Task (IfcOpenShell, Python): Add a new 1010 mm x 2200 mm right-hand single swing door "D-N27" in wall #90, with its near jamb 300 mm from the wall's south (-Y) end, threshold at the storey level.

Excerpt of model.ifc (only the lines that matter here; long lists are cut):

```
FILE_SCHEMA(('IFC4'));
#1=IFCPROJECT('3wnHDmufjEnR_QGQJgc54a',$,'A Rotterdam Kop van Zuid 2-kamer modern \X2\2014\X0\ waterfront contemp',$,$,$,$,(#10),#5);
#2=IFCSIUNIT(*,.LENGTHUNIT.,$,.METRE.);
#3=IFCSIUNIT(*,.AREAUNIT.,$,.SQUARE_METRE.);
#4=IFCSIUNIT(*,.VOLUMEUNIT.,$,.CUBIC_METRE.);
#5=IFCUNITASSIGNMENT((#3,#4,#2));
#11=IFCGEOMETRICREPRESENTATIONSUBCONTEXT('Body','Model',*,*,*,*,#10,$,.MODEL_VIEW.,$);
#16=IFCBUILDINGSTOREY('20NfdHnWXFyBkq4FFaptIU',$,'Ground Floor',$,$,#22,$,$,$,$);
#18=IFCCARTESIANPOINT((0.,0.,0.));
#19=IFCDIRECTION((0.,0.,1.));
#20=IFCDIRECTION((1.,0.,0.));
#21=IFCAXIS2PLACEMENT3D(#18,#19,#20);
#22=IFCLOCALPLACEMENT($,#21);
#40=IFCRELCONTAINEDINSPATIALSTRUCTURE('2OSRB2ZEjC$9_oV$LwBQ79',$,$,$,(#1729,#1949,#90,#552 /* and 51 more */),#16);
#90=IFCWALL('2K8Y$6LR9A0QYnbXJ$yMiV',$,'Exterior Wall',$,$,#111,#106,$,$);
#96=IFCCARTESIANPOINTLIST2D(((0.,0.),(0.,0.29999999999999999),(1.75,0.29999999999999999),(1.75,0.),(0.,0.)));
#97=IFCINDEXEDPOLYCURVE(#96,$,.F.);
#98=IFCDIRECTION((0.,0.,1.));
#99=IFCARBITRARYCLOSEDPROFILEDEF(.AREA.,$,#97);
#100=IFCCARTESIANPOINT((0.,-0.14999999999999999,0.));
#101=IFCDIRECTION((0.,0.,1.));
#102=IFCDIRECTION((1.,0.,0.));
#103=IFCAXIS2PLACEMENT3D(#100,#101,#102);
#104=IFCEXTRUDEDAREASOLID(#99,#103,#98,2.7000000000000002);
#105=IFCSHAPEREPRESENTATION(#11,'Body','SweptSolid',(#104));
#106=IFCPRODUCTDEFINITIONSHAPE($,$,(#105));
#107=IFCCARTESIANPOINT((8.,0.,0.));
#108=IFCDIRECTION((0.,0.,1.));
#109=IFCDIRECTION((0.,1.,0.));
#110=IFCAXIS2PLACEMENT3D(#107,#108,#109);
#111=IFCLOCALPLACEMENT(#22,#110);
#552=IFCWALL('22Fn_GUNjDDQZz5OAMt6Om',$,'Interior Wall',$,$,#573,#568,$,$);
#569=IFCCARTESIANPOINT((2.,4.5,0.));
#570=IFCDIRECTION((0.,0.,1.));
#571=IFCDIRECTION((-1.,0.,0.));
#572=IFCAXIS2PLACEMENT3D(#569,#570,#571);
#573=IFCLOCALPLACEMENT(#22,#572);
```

```python
import numpy as np
import ifcopenshell
import ifcopenshell.api.feature
import ifcopenshell.api.geometry
import ifcopenshell.api.root
import ifcopenshell.api.spatial
import ifcopenshell.geom
import ifcopenshell.util.element
import ifcopenshell.util.placement
import ifcopenshell.util.representation
import ifcopenshell.util.shape
import ifcopenshell.util.unit

model = ifcopenshell.open("model.ifc")
unit_scale = ifcopenshell.util.unit.calculate_unit_scale(model)
settings = ifcopenshell.geom.settings()


def volume(element):
    """Net volume in cubic metres, openings subtracted."""
    shape = ifcopenshell.geom.create_shape(settings, element)
    return ifcopenshell.util.shape.get_volume(shape.geometry)


wall = model.by_guid("2K8Y$6LR9A0QYnbXJ$yMiV")
storey = ifcopenshell.util.element.get_container(wall, ifc_class="IfcBuildingStorey")
context = ifcopenshell.util.representation.get_context(model, "Model", "Body", "MODEL_VIEW")
before = volume(wall)

width, height, from_end, sill = 1.01, 2.2, 0.3, 0.0  # metres

# The wall runs along its own X axis, and the end named is its -X end.
wall_shape = ifcopenshell.geom.create_shape(settings, wall)
x, y, z = ifcopenshell.util.shape.get_vertices(wall_shape.geometry).T
start = x.min() + from_end
face, thickness = float(y.min()), float(y.max() - y.min())
wall_matrix = ifcopenshell.util.placement.get_local_placement(wall.ObjectPlacement)
level = ifcopenshell.util.placement.get_local_placement(storey.ObjectPlacement)[2, 3]


def in_wall(x, y):
    """Placement at x, y metres in the wall's axes, at sill height."""
    matrix = wall_matrix.copy()
    matrix[:, 3] = wall_matrix @ np.array([x / unit_scale, y / unit_scale, 0.0, 1.0])
    matrix[2, 3] = level + sill / unit_scale
    return matrix


# Opening: a box that overshoots both wall faces by 50 mm.
opening = ifcopenshell.api.root.create_entity(model, ifc_class="IfcOpeningElement", predefined_type="OPENING")
box = ifcopenshell.api.geometry.add_wall_representation(
    model, context=context, length=width, height=height, thickness=thickness + 0.1
)
ifcopenshell.api.geometry.assign_representation(model, product=opening, representation=box)
ifcopenshell.api.geometry.edit_object_placement(model, product=opening, matrix=in_wall(start, face - 0.05), is_si=False)
ifcopenshell.api.feature.add_feature(model, feature=opening, element=wall)

door = ifcopenshell.api.root.create_entity(model, ifc_class="IfcDoor", name="D-N27", predefined_type="DOOR")
door.OverallWidth, door.OverallHeight = width / unit_scale, height / unit_scale
door.OperationType = "SINGLE_SWING_RIGHT"
body = ifcopenshell.api.geometry.add_door_representation(
    model,
    context=context,
    overall_width=door.OverallWidth,
    overall_height=door.OverallHeight,
    operation_type="SINGLE_SWING_RIGHT",
    lining_properties={"LiningDepth": thickness / unit_scale, "ThresholdDepth": thickness / unit_scale},
)
ifcopenshell.api.geometry.assign_representation(model, product=door, representation=body)
ifcopenshell.api.spatial.assign_container(model, products=[door], relating_structure=storey)
ifcopenshell.api.feature.add_filling(model, opening=opening, element=door)

# The lining spans the wall, so the door starts at the wall face.
ifcopenshell.api.geometry.edit_object_placement(model, product=door, matrix=in_wall(start, face), is_si=False)

after = volume(wall)

print(f"wall volume {before:.3f} -> {after:.3f} m3")

model.write("model_edited.ifc")
```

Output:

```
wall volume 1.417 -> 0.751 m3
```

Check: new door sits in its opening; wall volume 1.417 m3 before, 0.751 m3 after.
